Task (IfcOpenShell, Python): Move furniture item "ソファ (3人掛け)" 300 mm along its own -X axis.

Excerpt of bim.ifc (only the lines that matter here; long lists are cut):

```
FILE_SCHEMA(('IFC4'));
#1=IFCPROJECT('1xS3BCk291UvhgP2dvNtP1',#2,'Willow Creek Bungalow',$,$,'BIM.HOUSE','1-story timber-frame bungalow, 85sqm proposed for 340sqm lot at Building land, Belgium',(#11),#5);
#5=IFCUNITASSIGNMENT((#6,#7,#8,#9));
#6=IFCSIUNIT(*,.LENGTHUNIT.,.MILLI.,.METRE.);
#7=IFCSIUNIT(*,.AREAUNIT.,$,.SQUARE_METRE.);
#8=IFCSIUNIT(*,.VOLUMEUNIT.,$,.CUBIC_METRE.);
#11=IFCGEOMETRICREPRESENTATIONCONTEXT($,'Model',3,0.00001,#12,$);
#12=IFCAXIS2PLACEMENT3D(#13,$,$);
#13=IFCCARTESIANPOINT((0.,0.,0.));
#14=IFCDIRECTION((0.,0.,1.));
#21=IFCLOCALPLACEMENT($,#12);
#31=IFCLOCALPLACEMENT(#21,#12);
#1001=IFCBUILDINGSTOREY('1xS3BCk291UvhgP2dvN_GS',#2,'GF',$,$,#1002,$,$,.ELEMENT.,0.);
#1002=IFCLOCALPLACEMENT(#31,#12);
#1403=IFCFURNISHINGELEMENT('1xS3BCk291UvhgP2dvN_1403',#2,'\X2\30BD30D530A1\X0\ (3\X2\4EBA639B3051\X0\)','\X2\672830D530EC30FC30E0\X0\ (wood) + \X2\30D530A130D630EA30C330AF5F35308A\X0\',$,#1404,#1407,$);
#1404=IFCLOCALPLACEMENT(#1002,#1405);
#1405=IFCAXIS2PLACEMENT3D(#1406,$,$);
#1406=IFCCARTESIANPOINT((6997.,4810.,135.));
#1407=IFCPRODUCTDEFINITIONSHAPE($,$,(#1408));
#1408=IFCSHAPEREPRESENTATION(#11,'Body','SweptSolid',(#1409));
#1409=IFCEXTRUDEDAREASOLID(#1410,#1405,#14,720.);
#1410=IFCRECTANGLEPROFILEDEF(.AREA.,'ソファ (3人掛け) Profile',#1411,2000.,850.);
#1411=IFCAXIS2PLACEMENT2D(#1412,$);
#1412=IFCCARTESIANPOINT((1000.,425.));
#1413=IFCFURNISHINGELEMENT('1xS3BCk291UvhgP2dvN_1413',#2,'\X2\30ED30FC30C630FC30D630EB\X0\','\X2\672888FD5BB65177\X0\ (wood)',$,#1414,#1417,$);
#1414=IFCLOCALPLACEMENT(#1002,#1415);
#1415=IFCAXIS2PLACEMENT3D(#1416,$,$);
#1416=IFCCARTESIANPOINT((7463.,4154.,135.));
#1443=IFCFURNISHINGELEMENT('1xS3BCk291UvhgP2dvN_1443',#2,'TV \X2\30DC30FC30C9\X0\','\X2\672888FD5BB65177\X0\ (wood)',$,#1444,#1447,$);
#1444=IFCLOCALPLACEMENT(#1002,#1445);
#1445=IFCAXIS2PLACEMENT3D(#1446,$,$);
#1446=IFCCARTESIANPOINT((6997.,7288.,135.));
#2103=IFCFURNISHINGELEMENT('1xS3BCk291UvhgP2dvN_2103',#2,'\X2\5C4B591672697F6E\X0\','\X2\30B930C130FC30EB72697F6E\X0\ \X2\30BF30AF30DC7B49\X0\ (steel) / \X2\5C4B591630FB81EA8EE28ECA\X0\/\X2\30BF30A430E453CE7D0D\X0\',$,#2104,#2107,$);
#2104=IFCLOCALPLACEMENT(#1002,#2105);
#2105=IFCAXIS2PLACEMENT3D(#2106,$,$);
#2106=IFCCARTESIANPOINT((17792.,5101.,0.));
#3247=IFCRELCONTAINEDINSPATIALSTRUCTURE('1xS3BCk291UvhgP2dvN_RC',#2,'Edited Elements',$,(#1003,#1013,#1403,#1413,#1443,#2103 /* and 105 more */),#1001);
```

```python
import ifcopenshell
import ifcopenshell.api.geometry
import ifcopenshell.util.placement
import ifcopenshell.util.unit

model = ifcopenshell.open("bim.ifc")
unit_scale = ifcopenshell.util.unit.calculate_unit_scale(model)

item = model.by_guid("1xS3BCk291UvhgP2dvN_1403")
matrix = ifcopenshell.util.placement.get_local_placement(item.ObjectPlacement)
matrix[:3, 3] -= matrix[:3, 0] * 0.3 / unit_scale
ifcopenshell.api.geometry.edit_object_placement(model, product=item, matrix=matrix, is_si=False)

print(ifcopenshell.util.placement.get_local_placement(item.ObjectPlacement).round(3) + 0.0)

model.write("bim_v2.ifc")
```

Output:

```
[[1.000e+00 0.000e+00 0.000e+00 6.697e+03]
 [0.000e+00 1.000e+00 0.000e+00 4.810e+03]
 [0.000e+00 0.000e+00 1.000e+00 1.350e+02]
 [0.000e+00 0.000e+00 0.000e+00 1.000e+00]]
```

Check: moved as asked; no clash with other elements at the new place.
